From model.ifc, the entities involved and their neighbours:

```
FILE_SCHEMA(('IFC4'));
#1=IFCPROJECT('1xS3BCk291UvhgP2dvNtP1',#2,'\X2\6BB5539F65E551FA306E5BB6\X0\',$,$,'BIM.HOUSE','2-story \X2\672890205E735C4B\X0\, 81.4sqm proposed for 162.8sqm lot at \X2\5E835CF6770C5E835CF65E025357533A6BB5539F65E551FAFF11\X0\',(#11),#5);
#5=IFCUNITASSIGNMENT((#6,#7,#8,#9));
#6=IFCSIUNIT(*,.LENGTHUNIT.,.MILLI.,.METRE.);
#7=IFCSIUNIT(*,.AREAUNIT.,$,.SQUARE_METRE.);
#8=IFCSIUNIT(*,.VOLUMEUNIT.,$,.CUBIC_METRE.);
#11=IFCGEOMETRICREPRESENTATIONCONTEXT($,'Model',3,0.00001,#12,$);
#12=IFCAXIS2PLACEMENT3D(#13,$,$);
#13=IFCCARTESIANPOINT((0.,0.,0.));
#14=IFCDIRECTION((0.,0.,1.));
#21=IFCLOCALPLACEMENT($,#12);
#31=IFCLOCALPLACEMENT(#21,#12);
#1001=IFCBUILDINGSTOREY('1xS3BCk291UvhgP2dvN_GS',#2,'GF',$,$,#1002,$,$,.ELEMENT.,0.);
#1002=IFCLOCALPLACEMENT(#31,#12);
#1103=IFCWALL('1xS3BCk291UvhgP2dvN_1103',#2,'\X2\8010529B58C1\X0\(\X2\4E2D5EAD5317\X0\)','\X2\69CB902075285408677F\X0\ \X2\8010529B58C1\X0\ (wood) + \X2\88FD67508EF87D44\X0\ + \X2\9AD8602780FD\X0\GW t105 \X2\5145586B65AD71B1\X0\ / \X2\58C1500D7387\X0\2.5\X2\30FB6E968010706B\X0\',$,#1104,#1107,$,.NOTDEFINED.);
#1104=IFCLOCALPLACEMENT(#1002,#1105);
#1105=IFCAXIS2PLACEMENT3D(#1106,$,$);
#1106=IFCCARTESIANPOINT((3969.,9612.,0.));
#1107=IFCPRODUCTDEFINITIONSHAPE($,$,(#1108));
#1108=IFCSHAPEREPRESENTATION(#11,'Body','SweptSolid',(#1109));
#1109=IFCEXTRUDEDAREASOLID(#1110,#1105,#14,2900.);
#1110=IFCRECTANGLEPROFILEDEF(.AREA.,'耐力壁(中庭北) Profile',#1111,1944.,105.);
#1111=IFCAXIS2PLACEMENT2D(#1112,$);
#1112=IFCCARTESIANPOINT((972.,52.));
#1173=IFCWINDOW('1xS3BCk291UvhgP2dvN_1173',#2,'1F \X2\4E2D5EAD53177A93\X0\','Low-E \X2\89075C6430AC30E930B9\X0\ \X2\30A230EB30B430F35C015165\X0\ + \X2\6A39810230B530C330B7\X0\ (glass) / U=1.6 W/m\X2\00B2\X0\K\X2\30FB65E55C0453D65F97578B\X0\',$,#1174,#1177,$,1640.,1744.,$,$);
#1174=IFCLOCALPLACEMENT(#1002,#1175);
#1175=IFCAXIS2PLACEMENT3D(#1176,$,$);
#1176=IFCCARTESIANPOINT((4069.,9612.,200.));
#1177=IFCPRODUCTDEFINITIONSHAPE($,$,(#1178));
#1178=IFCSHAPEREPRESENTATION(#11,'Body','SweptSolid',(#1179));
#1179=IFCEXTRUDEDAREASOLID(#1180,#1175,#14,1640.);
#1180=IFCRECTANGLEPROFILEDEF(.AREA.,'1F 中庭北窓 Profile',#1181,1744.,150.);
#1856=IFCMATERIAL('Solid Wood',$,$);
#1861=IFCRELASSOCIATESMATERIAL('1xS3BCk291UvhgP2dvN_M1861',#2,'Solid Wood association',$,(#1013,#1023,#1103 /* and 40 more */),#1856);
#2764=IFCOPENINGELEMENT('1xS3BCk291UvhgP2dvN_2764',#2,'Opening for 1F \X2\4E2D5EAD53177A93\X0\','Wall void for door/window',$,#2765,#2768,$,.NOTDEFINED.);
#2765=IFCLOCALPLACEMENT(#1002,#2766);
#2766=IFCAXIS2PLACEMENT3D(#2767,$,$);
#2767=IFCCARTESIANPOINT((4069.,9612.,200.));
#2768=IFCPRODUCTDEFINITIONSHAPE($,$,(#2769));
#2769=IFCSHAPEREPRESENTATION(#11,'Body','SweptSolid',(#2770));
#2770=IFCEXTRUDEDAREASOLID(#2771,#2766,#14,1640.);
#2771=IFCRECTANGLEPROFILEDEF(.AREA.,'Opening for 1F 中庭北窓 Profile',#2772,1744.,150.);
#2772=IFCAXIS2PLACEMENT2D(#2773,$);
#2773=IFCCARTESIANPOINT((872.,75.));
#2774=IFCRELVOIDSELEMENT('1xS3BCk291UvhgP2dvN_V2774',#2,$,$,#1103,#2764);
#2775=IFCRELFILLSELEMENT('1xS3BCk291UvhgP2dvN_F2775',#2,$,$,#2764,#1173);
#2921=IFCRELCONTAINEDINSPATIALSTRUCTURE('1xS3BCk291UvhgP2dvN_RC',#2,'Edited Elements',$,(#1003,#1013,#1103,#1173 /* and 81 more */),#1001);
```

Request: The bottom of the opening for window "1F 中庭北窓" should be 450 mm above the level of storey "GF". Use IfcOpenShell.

```python
import numpy as np
import ifcopenshell
import ifcopenshell.api.geometry
import ifcopenshell.geom
import ifcopenshell.util.element
import ifcopenshell.util.placement
import ifcopenshell.util.shape
import ifcopenshell.util.unit

model = ifcopenshell.open("model.ifc")
unit_scale = ifcopenshell.util.unit.calculate_unit_scale(model)

window = model.by_guid("1xS3BCk291UvhgP2dvN_1173")
opening = window.FillsVoids[0].RelatingOpeningElement
storey = ifcopenshell.util.element.get_container(window, ifc_class="IfcBuildingStorey")
level = ifcopenshell.util.placement.get_local_placement(storey.ObjectPlacement)[2, 3]

# The opening's origin need not be at the sill, so measure its lowest point.
shape = ifcopenshell.geom.create_shape(ifcopenshell.geom.settings(), opening)
bottom = ifcopenshell.util.shape.get_shape_bottom_elevation(shape, shape.geometry) / unit_scale
dz = level + 0.45 / unit_scale - bottom

shift = np.array([0.0, 0.0, dz])
# The window is not placed relative to its opening, so move both.
for product in (opening, window):
    matrix = ifcopenshell.util.placement.get_local_placement(product.ObjectPlacement)
    matrix[:3, 3] += shift
    ifcopenshell.api.geometry.edit_object_placement(model, product=product, matrix=matrix, is_si=False)

print(f"moved by {dz * unit_scale:+.3f} m")

model.write("model_v2.ifc")
```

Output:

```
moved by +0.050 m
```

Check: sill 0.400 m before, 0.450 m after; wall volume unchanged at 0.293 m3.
